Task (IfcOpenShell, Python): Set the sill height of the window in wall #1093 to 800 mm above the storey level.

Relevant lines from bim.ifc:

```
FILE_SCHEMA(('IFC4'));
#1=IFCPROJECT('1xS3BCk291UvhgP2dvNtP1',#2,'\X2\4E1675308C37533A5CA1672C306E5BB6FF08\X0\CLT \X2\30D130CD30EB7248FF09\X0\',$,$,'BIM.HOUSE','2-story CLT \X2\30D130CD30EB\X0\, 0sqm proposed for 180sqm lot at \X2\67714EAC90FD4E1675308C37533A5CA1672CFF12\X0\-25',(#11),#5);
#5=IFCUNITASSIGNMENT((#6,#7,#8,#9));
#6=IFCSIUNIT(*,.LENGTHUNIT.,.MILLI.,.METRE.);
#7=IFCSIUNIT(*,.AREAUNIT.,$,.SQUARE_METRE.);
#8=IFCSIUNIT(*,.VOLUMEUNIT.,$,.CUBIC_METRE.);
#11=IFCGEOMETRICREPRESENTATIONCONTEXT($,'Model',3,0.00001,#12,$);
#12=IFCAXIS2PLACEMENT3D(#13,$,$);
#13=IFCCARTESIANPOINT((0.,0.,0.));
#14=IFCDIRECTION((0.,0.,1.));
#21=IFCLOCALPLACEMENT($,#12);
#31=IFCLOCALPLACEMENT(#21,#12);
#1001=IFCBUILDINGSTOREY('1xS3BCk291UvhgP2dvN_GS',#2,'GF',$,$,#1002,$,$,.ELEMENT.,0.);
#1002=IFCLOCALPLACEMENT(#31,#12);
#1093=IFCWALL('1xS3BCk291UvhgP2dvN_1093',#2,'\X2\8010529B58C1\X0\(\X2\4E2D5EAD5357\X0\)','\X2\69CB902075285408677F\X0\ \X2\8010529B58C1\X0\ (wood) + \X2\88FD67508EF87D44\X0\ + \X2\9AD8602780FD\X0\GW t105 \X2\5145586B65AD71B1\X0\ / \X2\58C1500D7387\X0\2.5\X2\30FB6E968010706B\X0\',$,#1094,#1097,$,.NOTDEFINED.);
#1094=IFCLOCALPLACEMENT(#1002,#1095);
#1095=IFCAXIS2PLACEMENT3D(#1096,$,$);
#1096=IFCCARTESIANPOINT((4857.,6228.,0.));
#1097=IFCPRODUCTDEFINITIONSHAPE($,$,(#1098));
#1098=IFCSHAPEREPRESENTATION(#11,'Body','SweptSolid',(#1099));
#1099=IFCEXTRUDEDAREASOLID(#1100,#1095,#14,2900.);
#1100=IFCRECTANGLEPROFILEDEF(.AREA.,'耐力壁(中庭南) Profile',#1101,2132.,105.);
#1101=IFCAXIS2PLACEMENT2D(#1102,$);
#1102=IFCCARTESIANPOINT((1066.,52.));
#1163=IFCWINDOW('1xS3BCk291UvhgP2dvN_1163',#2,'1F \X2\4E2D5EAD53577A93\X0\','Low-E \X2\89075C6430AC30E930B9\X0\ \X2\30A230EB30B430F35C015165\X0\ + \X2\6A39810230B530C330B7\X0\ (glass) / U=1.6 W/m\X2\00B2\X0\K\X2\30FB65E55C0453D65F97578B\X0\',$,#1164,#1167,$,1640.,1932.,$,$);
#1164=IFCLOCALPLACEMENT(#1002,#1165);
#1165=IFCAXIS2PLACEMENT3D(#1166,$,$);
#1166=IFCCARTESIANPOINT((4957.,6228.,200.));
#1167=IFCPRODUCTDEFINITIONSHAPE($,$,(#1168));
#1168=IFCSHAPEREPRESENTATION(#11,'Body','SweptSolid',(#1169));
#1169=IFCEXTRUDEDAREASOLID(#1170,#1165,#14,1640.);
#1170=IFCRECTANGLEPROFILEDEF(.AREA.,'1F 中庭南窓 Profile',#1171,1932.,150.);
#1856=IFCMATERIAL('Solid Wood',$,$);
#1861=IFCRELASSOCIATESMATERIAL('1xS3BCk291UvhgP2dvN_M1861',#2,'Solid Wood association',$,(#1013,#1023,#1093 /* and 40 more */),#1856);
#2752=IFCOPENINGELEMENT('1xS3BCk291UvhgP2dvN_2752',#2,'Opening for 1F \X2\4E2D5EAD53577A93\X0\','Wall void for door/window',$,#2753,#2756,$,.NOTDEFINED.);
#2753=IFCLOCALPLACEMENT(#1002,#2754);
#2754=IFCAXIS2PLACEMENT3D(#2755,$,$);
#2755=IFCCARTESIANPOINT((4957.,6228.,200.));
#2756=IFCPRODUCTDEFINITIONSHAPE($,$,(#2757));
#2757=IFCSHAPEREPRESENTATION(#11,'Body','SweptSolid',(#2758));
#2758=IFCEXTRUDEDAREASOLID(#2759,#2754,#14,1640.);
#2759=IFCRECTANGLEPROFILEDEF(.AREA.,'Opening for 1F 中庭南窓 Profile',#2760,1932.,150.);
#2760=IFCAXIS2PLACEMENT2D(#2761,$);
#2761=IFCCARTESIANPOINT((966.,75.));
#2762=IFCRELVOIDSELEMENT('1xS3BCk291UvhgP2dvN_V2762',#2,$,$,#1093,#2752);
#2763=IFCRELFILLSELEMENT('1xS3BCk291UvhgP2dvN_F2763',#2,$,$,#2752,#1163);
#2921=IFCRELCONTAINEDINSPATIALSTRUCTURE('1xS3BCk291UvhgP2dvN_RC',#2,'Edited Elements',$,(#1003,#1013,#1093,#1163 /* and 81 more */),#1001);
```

```python
import numpy as np
import ifcopenshell
import ifcopenshell.api.geometry
import ifcopenshell.geom
import ifcopenshell.util.element
import ifcopenshell.util.placement
import ifcopenshell.util.shape
import ifcopenshell.util.unit

model = ifcopenshell.open("bim.ifc")
unit_scale = ifcopenshell.util.unit.calculate_unit_scale(model)

window = model.by_guid("1xS3BCk291UvhgP2dvN_1163")
opening = window.FillsVoids[0].RelatingOpeningElement
storey = ifcopenshell.util.element.get_container(window, ifc_class="IfcBuildingStorey")
level = ifcopenshell.util.placement.get_local_placement(storey.ObjectPlacement)[2, 3]

# The opening's origin need not be at the sill, so measure its lowest point.
shape = ifcopenshell.geom.create_shape(ifcopenshell.geom.settings(), opening)
bottom = ifcopenshell.util.shape.get_shape_bottom_elevation(shape, shape.geometry) / unit_scale
dz = level + 0.8 / unit_scale - bottom

shift = np.array([0.0, 0.0, dz])
# The window is not placed relative to its opening, so move both.
for product in (opening, window):
    matrix = ifcopenshell.util.placement.get_local_placement(product.ObjectPlacement)
    matrix[:3, 3] += shift
    ifcopenshell.api.geometry.edit_object_placement(model, product=product, matrix=matrix, is_si=False)

print(f"moved by {dz * unit_scale:+.3f} m")

model.write("bim_rev.ifc")
```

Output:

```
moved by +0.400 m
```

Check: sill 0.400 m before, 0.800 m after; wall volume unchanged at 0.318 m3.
